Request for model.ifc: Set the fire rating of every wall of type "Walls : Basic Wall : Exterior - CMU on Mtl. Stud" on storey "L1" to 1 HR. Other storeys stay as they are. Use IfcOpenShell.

First a look at what the model holds.

```python
import ifcopenshell
import ifcopenshell.util.element

model = ifcopenshell.open("model.ifc")
print(model.schema)
storey = next(s for s in model.by_type("IfcBuildingStorey") if s.Name == "L1")
walls = [e for e in ifcopenshell.util.element.get_decomposition(storey) if e.is_a("IfcWall")]
seen = {}
for e in walls:
    element_type = ifcopenshell.util.element.get_type(e)
    key = (element_type.Name if element_type != e and element_type else None, ifcopenshell.util.element.get_pset(e, "Pset_WallCommon", "FireRating"))
    seen[key] = seen.get(key, 0) + 1
for (name, value), count in sorted(seen.items(), key=str):
    print(count, "x", name, "|", value)
```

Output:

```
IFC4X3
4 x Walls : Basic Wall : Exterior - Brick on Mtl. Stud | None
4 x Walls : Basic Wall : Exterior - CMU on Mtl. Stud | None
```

```python
import ifcopenshell
import ifcopenshell.api.pset
import ifcopenshell.util.element

model = ifcopenshell.open("model.ifc")

storey = next(s for s in model.by_type("IfcBuildingStorey") if s.Name == "L1")
walls = [e for e in ifcopenshell.util.element.get_decomposition(storey) if e.is_a("IfcWall")]

count = 0
for e in walls:
    element_type = ifcopenshell.util.element.get_type(e)
    if element_type in (None, e) or element_type.Name != "Walls : Basic Wall : Exterior - CMU on Mtl. Stud":
        continue
    # add_pset returns the element's existing set when there is one.
    pset = ifcopenshell.api.pset.add_pset(model, product=e, name="Pset_WallCommon")
    ifcopenshell.api.pset.edit_pset(model, pset=pset, properties={"FireRating": "1 HR"})
    count += 1

print(count, "walls updated")

model.write("model_rev.ifc")
```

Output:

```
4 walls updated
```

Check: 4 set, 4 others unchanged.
